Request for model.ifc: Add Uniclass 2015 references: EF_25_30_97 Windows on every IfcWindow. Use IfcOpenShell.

First a look at what the model holds.

```python
import ifcopenshell

model = ifcopenshell.open("model.ifc")
print(model.schema)
print("classifications:", [c.Name for c in model.by_type("IfcClassification")])
for ifc_class in ("IfcDoor", "IfcRoof", "IfcStair", "IfcWall", "IfcWindow"):
    print(ifc_class, len(model.by_type(ifc_class)))
```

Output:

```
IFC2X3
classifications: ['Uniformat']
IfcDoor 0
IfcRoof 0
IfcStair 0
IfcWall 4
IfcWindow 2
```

```python
import ifcopenshell
import ifcopenshell.api.classification

model = ifcopenshell.open("model.ifc")

# IFC2X3 requires Source and Edition and has no link from the project to the system.
system = model.create_entity("IfcClassification", Source="NBS", Edition="2015", Name="Uniclass 2015")

codes = {
    "IfcWindow": ("EF_25_30_97", "Windows"),
}
for ifc_class, (code, name) in codes.items():
    products = model.by_type(ifc_class)
    ifcopenshell.api.classification.add_reference(
        model, products=products, classification=system, identification=code, name=name
    )
    print(code, len(products))

model.write("model_edited.ifc")
```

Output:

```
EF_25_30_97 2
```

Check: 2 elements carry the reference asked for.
